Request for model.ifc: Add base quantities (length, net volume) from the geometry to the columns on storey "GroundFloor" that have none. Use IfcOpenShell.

First a look at what the model holds.

```python
import ifcopenshell
import ifcopenshell.util.element
import ifcopenshell.util.unit

model = ifcopenshell.open("model.ifc")
print(model.schema)
for unit_type in ("LENGTHUNIT", "AREAUNIT", "VOLUMEUNIT"):
    print(unit_type, ifcopenshell.util.unit.calculate_unit_scale(model, unit_type))
storey = next(s for s in model.by_type("IfcBuildingStorey") if s.Name == "GroundFloor")
columns = [e for e in ifcopenshell.util.element.get_decomposition(storey) if e.is_a("IfcColumn")]
for e in sorted(columns, key=lambda e: e.id()):
    print(e.id(), e.is_a(), e.Name, list(ifcopenshell.util.element.get_psets(e, qtos_only=True)), sep=" | ")
```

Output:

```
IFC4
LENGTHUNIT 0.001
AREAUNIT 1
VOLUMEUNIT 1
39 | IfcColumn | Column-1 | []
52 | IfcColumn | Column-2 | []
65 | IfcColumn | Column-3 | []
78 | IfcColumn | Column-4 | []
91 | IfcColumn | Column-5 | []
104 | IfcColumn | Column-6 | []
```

```python
import ifcopenshell
import ifcopenshell.api.pset
import ifcopenshell.geom
import ifcopenshell.util.element
import ifcopenshell.util.shape
import ifcopenshell.util.unit

model = ifcopenshell.open("model.ifc")
unit_scale = ifcopenshell.util.unit.calculate_unit_scale(model)
volume_scale = ifcopenshell.util.unit.calculate_unit_scale(model, "VOLUMEUNIT")
settings = ifcopenshell.geom.settings()

storey = next(s for s in model.by_type("IfcBuildingStorey") if s.Name == "GroundFloor")
columns = [e for e in ifcopenshell.util.element.get_decomposition(storey) if e.is_a("IfcColumn")]

for e in sorted(columns, key=lambda e: e.id()):
    if ifcopenshell.util.element.get_psets(e, qtos_only=True, should_inherit=False):
        continue
    # Geometry comes back in metres, in the element's own axes.
    shape = ifcopenshell.geom.create_shape(settings, e)
    values = {
        "Length": ifcopenshell.util.shape.get_z(shape.geometry) / unit_scale,
        "NetVolume": ifcopenshell.util.shape.get_volume(shape.geometry) / volume_scale,
    }
    qto = ifcopenshell.api.pset.add_qto(model, product=e, name="Qto_ColumnBaseQuantities")
    ifcopenshell.api.pset.edit_qto(model, qto=qto, properties=values)
    print(e.id(), {k: round(v, 3) for k, v in values.items()})

model.write("model_updated.ifc")
```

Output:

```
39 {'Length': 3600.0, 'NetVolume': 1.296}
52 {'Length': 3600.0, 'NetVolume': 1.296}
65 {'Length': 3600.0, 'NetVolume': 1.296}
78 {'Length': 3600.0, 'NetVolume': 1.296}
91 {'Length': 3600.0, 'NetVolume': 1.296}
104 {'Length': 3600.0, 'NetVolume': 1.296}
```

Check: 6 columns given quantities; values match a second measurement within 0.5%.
